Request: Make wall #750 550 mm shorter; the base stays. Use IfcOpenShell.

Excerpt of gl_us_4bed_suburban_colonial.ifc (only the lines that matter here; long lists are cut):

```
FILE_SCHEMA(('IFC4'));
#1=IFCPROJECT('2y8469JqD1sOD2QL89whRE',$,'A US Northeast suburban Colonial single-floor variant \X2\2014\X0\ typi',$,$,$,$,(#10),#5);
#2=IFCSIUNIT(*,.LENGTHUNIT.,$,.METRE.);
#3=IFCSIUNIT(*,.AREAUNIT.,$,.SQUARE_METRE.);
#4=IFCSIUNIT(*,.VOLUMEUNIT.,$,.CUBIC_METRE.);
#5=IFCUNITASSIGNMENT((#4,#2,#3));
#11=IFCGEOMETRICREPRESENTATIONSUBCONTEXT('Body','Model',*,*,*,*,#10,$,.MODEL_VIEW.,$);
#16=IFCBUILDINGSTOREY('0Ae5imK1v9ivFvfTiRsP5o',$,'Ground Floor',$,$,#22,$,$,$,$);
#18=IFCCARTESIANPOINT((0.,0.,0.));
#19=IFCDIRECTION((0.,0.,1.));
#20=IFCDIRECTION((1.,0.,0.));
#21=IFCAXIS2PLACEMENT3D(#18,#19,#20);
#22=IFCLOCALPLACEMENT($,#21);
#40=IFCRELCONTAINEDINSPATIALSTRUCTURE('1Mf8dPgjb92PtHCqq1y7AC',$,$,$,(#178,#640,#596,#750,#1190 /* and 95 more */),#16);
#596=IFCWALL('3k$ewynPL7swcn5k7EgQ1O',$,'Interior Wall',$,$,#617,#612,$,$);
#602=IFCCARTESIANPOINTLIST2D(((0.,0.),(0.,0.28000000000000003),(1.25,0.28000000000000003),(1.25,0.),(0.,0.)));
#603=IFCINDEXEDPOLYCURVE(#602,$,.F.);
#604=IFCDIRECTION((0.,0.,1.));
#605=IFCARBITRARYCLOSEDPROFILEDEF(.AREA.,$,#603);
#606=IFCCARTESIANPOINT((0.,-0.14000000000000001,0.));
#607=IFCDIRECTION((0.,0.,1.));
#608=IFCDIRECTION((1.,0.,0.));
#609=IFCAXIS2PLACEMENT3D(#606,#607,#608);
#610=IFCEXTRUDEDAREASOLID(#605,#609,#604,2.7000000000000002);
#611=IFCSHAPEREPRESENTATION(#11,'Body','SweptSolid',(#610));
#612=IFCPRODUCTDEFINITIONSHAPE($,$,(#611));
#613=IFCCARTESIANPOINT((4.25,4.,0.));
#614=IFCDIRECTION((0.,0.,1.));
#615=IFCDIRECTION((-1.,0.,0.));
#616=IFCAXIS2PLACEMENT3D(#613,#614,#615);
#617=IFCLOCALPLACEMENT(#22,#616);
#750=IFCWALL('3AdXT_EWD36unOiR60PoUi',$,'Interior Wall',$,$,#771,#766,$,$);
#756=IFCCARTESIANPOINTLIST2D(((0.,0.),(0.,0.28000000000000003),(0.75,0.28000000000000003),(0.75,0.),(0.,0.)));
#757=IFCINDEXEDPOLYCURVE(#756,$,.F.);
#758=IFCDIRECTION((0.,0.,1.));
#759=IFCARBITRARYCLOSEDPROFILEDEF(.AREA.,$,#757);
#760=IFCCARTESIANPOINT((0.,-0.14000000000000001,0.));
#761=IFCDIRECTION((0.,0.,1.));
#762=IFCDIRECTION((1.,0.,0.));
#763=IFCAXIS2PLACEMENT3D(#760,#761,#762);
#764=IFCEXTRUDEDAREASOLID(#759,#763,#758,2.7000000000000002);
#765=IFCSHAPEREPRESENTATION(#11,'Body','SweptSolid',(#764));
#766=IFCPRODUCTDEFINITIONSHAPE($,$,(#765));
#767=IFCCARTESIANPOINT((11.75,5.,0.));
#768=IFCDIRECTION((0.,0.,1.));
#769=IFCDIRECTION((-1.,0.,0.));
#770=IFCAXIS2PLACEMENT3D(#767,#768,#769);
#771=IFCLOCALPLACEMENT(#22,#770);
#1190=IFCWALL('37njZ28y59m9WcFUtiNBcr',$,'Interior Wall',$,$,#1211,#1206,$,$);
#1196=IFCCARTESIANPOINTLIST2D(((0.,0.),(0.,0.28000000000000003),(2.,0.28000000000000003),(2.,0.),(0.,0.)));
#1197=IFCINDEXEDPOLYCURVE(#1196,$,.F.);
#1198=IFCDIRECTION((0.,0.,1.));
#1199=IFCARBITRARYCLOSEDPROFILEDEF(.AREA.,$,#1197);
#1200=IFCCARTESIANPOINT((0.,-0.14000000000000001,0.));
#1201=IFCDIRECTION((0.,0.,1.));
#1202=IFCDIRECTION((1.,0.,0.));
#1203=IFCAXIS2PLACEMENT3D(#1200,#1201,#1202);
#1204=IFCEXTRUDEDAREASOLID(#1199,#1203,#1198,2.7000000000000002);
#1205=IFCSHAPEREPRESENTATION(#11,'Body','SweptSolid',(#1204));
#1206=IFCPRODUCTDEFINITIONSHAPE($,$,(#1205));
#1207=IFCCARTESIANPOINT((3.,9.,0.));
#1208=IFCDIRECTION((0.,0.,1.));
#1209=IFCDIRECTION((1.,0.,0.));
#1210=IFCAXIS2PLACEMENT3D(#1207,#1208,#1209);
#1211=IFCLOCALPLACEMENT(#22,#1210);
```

```python
import ifcopenshell
import ifcopenshell.geom
import ifcopenshell.util.representation
import ifcopenshell.util.shape
import ifcopenshell.util.unit

model = ifcopenshell.open("gl_us_4bed_suburban_colonial.ifc")
unit_scale = ifcopenshell.util.unit.calculate_unit_scale(model)
settings = ifcopenshell.geom.settings()


def volume(element):
    """Net volume in cubic metres, openings subtracted."""
    shape = ifcopenshell.geom.create_shape(settings, element)
    return ifcopenshell.util.shape.get_volume(shape.geometry)


wall = model.by_guid("3AdXT_EWD36unOiR60PoUi")
before = volume(wall)

body = ifcopenshell.util.representation.get_representation(wall, "Model", "Body")
solid = body.Items[0]
old_height = solid.Depth
solid.Depth -= 0.55 / unit_scale
after = volume(wall)

print(f"height {old_height:g} -> {solid.Depth:g}, volume {before:.3f} -> {after:.3f} m3")

model.write("gl_us_4bed_suburban_colonial_edited.ifc")
```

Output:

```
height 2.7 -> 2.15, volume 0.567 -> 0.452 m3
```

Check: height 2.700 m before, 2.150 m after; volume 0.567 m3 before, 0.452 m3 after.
